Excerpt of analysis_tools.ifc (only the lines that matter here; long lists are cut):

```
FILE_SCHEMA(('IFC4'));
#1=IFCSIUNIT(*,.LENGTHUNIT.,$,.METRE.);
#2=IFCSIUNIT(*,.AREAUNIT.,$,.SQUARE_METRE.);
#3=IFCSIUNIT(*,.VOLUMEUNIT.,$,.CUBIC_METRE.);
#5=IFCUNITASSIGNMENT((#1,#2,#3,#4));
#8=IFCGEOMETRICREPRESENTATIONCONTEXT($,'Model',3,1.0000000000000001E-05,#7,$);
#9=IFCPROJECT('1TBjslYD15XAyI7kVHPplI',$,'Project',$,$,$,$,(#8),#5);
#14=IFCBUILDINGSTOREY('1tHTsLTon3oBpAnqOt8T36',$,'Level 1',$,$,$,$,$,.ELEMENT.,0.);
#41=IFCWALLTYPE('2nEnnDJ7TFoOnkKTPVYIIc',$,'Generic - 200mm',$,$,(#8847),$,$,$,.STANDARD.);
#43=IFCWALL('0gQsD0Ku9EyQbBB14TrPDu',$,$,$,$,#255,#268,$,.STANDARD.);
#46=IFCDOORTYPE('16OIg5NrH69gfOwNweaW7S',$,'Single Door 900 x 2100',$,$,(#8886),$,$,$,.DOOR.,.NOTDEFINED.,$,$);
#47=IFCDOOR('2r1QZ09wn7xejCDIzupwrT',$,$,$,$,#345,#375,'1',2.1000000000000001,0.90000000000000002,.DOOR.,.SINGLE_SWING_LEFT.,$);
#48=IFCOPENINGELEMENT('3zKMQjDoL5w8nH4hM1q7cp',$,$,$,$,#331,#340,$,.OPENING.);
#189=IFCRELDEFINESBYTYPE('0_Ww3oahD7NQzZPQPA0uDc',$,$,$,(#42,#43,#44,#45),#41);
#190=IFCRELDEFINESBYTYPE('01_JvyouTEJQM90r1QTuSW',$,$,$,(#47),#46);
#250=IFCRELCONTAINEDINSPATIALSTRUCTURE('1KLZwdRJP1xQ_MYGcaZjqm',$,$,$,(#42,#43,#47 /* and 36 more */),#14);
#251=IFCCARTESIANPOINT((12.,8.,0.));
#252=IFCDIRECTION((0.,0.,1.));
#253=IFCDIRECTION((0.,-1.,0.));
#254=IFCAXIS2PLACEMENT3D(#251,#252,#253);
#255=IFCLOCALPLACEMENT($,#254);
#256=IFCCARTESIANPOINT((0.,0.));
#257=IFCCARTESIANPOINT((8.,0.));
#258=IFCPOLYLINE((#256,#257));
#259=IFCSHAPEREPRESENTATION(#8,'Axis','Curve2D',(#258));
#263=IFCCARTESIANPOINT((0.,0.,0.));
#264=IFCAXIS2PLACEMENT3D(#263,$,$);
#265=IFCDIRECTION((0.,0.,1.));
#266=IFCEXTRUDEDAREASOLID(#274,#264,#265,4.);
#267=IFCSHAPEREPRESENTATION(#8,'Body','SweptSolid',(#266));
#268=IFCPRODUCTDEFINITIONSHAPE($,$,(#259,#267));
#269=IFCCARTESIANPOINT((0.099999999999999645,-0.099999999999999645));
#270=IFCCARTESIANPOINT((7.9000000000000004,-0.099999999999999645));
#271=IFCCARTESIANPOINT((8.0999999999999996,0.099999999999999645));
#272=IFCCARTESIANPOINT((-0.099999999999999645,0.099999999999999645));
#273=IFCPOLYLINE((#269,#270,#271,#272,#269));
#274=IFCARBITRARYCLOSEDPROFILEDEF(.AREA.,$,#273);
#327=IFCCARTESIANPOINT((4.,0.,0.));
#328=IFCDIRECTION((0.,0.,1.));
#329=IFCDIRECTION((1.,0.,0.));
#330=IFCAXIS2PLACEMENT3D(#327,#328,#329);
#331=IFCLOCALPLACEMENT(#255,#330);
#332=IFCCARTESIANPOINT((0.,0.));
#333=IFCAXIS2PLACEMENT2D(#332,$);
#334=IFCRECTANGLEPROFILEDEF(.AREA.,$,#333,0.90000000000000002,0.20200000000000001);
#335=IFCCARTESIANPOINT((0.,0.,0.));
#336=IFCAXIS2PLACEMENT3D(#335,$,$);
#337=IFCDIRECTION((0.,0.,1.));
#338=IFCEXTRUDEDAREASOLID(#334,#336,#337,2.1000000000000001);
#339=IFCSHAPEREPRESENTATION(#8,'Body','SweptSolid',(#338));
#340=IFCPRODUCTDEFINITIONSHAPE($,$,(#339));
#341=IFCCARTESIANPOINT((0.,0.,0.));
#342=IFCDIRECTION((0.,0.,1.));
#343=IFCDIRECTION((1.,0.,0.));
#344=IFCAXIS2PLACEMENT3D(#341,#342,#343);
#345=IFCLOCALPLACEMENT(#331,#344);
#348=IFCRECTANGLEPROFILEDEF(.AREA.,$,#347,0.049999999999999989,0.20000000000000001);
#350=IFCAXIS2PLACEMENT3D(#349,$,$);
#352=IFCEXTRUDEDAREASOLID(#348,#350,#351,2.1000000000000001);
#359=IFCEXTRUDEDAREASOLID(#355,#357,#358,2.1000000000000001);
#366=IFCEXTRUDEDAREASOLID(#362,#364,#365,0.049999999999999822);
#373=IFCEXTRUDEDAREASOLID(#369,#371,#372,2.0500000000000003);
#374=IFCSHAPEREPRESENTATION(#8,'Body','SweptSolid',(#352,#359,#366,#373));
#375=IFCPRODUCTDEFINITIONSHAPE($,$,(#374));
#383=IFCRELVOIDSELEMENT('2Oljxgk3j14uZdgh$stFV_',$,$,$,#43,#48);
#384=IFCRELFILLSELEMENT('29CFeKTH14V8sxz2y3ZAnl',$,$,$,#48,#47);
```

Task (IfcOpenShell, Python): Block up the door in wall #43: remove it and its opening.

```python
import ifcopenshell
import ifcopenshell.api.feature
import ifcopenshell.api.root
import ifcopenshell.geom
import ifcopenshell.util.shape

model = ifcopenshell.open("analysis_tools.ifc")
settings = ifcopenshell.geom.settings()


def volume(element):
    """Net volume in cubic metres, openings subtracted."""
    shape = ifcopenshell.geom.create_shape(settings, element)
    return ifcopenshell.util.shape.get_volume(shape.geometry)


door = model.by_guid("2r1QZ09wn7xejCDIzupwrT")
opening = door.FillsVoids[0].RelatingOpeningElement
wall = opening.VoidsElements[0].RelatingBuildingElement
before = volume(wall)

ifcopenshell.api.root.remove_product(model, product=door)
ifcopenshell.api.feature.remove_feature(model, feature=opening)

after = volume(wall)

print(f"wall volume {before:.3f} -> {after:.3f} m3")

model.write("analysis_tools_rev.ifc")
```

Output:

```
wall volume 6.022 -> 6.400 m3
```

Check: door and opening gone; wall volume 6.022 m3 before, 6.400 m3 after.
